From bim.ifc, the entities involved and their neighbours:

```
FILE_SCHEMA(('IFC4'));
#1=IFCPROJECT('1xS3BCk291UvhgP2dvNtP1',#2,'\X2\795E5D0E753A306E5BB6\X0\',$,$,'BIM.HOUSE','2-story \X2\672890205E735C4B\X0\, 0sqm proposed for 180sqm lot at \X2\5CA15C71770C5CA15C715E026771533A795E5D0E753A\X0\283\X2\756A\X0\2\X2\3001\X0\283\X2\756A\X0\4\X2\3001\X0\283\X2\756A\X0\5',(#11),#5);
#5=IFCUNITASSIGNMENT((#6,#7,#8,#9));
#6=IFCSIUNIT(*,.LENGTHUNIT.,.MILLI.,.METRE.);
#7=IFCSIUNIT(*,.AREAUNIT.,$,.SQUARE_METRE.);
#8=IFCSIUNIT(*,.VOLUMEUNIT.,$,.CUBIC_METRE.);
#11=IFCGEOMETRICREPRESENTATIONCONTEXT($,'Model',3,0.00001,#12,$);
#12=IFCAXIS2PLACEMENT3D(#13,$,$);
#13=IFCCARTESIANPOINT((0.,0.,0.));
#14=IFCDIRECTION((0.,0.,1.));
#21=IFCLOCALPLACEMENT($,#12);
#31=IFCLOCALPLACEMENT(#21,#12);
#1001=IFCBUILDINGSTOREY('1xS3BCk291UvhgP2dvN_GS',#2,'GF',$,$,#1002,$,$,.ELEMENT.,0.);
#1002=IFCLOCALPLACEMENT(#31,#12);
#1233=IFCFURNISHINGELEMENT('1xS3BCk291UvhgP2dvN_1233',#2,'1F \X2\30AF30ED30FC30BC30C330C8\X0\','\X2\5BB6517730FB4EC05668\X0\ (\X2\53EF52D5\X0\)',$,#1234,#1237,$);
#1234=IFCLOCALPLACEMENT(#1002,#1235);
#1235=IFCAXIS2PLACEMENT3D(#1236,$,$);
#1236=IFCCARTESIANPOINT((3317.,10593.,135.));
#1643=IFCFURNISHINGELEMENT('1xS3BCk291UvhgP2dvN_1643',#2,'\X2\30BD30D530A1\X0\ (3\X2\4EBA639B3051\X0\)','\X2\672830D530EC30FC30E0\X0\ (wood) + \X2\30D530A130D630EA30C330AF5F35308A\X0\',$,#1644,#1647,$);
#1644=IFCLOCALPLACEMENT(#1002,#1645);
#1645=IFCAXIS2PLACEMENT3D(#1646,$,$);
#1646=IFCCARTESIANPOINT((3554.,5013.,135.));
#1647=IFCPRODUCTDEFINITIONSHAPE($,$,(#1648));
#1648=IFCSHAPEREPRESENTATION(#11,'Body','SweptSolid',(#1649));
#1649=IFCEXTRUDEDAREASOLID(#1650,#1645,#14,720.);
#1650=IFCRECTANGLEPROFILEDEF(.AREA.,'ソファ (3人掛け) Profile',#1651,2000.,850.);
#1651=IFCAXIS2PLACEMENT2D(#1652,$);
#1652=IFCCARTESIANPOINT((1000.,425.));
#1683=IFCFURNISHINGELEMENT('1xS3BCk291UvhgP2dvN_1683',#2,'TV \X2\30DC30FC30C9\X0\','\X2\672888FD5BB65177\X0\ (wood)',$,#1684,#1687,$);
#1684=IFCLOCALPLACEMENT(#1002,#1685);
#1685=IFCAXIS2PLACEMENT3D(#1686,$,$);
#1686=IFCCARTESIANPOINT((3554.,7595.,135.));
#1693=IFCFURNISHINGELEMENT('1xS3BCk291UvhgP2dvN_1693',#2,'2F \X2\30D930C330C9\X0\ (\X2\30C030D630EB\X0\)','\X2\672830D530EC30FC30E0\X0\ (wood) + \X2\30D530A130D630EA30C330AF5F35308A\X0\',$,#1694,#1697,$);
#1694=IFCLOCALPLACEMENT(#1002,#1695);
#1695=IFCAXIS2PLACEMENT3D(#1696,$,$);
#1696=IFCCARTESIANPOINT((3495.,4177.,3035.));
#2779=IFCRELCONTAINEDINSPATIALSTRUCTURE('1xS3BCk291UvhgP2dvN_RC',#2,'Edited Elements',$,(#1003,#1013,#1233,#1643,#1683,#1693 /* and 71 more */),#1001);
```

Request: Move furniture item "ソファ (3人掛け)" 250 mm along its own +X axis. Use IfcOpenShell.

```python
import ifcopenshell
import ifcopenshell.api.geometry
import ifcopenshell.util.placement
import ifcopenshell.util.unit

model = ifcopenshell.open("bim.ifc")
unit_scale = ifcopenshell.util.unit.calculate_unit_scale(model)

item = model.by_guid("1xS3BCk291UvhgP2dvN_1643")
matrix = ifcopenshell.util.placement.get_local_placement(item.ObjectPlacement)
matrix[:3, 3] += matrix[:3, 0] * 0.25 / unit_scale
ifcopenshell.api.geometry.edit_object_placement(model, product=item, matrix=matrix, is_si=False)

print(ifcopenshell.util.placement.get_local_placement(item.ObjectPlacement).round(3) + 0.0)

model.write("bim_v2.ifc")
```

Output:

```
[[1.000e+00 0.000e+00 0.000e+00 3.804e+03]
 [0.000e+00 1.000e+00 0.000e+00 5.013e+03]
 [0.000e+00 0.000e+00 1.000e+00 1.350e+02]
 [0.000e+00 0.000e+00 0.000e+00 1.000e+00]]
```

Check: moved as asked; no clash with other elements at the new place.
